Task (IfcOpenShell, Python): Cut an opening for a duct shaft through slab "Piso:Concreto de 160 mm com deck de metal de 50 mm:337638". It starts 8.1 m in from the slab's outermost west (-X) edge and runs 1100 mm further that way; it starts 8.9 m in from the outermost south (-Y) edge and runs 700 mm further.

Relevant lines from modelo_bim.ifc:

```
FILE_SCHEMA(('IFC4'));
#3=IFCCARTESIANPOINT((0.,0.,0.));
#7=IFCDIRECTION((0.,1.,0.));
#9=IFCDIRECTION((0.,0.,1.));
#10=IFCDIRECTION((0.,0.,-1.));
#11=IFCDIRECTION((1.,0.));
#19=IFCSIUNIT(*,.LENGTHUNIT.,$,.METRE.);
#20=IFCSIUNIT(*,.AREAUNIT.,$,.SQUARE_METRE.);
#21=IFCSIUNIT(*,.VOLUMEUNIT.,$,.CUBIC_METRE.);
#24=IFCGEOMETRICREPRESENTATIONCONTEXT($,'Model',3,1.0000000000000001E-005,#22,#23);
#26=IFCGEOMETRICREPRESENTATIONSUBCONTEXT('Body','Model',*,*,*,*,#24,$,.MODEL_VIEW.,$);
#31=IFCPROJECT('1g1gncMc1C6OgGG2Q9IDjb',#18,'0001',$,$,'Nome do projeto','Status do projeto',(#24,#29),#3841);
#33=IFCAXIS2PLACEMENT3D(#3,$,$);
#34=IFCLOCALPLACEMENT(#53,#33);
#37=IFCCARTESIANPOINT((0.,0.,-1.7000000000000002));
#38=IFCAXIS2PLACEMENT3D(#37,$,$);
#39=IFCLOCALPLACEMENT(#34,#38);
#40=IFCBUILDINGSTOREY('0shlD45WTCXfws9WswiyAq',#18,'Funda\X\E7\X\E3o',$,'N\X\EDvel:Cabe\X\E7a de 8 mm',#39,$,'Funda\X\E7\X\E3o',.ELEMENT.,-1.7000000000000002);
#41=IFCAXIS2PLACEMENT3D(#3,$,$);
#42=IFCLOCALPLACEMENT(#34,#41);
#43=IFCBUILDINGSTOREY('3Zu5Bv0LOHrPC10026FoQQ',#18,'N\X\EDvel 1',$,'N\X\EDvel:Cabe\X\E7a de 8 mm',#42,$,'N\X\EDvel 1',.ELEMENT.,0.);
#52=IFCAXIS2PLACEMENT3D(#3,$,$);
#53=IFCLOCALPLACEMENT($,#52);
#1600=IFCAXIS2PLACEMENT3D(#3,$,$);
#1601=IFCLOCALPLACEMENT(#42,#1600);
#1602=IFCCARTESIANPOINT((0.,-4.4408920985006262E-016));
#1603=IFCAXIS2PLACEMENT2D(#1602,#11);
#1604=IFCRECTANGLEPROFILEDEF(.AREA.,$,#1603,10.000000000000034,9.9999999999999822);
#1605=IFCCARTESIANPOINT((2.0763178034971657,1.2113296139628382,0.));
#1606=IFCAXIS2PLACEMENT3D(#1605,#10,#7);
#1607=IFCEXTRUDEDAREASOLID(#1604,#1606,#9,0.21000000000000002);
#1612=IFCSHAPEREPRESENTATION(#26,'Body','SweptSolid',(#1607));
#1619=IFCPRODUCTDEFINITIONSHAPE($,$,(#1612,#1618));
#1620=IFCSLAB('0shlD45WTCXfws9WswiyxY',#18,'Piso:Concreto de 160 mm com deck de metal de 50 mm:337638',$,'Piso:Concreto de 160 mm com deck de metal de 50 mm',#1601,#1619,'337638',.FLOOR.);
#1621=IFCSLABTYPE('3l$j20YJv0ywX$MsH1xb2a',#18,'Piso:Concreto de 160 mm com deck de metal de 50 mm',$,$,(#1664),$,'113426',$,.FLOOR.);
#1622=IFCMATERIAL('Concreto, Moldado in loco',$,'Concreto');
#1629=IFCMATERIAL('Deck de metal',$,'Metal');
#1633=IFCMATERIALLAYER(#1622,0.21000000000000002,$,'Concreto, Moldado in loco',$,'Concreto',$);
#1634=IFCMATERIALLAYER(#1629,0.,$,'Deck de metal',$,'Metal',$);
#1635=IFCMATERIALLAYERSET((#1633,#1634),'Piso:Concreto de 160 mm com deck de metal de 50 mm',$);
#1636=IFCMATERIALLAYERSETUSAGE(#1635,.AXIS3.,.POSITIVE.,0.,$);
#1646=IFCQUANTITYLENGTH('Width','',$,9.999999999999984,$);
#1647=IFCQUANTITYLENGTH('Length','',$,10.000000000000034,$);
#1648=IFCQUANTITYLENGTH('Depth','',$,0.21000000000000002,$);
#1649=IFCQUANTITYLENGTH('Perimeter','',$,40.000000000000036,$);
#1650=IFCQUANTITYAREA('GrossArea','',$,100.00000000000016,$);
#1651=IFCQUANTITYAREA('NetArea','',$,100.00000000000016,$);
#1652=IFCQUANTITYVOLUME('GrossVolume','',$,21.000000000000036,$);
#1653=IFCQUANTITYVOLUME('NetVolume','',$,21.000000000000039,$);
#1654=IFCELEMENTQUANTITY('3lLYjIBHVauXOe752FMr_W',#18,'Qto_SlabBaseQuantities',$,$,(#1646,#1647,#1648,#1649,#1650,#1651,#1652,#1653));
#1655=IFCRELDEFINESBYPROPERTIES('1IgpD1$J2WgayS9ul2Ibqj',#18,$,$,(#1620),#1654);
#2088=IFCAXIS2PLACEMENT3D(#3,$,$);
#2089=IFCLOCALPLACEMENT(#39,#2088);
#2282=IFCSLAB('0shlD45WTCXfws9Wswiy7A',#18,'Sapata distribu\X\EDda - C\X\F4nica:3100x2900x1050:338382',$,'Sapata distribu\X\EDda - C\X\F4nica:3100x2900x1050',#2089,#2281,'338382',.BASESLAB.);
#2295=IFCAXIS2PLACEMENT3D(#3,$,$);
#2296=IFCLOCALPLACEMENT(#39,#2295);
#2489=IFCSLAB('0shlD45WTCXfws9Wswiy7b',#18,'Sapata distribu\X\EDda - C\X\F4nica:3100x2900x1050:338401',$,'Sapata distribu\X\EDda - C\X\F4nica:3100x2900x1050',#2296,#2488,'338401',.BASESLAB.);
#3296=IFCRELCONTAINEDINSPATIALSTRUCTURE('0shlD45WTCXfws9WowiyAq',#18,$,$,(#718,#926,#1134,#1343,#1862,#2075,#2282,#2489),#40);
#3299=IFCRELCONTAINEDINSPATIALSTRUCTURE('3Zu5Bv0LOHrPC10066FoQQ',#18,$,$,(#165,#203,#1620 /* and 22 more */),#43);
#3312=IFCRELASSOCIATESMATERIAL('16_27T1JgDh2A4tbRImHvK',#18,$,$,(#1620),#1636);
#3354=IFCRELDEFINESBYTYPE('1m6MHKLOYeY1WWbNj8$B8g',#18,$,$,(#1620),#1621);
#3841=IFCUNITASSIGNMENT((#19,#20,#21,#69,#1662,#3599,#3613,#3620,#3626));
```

```python
import numpy as np
import ifcopenshell
import ifcopenshell.api.feature
import ifcopenshell.api.geometry
import ifcopenshell.api.pset
import ifcopenshell.api.root
import ifcopenshell.geom
import ifcopenshell.util.element
import ifcopenshell.util.placement
import ifcopenshell.util.representation
import ifcopenshell.util.shape
import ifcopenshell.util.unit

model = ifcopenshell.open("modelo_bim.ifc")
unit_scale = ifcopenshell.util.unit.calculate_unit_scale(model)
area_scale = ifcopenshell.util.unit.calculate_unit_scale(model, "AREAUNIT")
volume_scale = ifcopenshell.util.unit.calculate_unit_scale(model, "VOLUMEUNIT")
settings = ifcopenshell.geom.settings()


def volume(element):
    """Net volume in cubic metres, openings subtracted."""
    shape = ifcopenshell.geom.create_shape(settings, element)
    return ifcopenshell.util.shape.get_volume(shape.geometry)


slab = model.by_guid("0shlD45WTCXfws9WswiyxY")
before = volume(slab)

# Extent in the slab's own axes, in metres. The edges named are its -X and -Y sides.
slab_shape = ifcopenshell.geom.create_shape(settings, slab)
vertices = ifcopenshell.util.shape.get_vertices(slab_shape.geometry)
x_min, y_min, bottom = vertices.min(axis=0)
top = vertices[:, 2].max()

opening = ifcopenshell.api.root.create_entity(model, ifc_class="IfcOpeningElement", name="Duct shaft opening", predefined_type="OPENING")
context = ifcopenshell.util.representation.get_context(model, "Model", "Body", "MODEL_VIEW")
width, depth = 1.1, 0.7
outline = [(0.0, 0.0), (width, 0.0), (width, depth), (0.0, depth), (0.0, 0.0)]
# Overshoot both faces by 50 mm so the cut is clean.
shape = ifcopenshell.api.geometry.add_slab_representation(
    model, context=context, depth=top - bottom + 0.1, polyline=outline
)
ifcopenshell.api.geometry.assign_representation(model, product=opening, representation=shape)

matrix = ifcopenshell.util.placement.get_local_placement(slab.ObjectPlacement)
matrix[:, 3] = matrix @ np.append(np.array([x_min + 8.1, y_min + 8.9, bottom - 0.05]) / unit_scale, 1.0)
ifcopenshell.api.geometry.edit_object_placement(model, product=opening, matrix=matrix, is_si=False)
ifcopenshell.api.feature.add_feature(model, feature=opening, element=slab)

after = volume(slab)

# Update the slab's stored quantities.
qto = model.by_id(ifcopenshell.util.element.get_pset(slab, "Qto_SlabBaseQuantities", should_inherit=False)["id"])
ifcopenshell.api.pset.edit_qto(model, qto=qto, properties={
    "NetArea": after / (top - bottom) / area_scale,
    "NetVolume": after / volume_scale,
})

print(f"slab volume {before:.3f} -> {after:.3f} m3")

model.write("modelo_bim_v2.ifc")
```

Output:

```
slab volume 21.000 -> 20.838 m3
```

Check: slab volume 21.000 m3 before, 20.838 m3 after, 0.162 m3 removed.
